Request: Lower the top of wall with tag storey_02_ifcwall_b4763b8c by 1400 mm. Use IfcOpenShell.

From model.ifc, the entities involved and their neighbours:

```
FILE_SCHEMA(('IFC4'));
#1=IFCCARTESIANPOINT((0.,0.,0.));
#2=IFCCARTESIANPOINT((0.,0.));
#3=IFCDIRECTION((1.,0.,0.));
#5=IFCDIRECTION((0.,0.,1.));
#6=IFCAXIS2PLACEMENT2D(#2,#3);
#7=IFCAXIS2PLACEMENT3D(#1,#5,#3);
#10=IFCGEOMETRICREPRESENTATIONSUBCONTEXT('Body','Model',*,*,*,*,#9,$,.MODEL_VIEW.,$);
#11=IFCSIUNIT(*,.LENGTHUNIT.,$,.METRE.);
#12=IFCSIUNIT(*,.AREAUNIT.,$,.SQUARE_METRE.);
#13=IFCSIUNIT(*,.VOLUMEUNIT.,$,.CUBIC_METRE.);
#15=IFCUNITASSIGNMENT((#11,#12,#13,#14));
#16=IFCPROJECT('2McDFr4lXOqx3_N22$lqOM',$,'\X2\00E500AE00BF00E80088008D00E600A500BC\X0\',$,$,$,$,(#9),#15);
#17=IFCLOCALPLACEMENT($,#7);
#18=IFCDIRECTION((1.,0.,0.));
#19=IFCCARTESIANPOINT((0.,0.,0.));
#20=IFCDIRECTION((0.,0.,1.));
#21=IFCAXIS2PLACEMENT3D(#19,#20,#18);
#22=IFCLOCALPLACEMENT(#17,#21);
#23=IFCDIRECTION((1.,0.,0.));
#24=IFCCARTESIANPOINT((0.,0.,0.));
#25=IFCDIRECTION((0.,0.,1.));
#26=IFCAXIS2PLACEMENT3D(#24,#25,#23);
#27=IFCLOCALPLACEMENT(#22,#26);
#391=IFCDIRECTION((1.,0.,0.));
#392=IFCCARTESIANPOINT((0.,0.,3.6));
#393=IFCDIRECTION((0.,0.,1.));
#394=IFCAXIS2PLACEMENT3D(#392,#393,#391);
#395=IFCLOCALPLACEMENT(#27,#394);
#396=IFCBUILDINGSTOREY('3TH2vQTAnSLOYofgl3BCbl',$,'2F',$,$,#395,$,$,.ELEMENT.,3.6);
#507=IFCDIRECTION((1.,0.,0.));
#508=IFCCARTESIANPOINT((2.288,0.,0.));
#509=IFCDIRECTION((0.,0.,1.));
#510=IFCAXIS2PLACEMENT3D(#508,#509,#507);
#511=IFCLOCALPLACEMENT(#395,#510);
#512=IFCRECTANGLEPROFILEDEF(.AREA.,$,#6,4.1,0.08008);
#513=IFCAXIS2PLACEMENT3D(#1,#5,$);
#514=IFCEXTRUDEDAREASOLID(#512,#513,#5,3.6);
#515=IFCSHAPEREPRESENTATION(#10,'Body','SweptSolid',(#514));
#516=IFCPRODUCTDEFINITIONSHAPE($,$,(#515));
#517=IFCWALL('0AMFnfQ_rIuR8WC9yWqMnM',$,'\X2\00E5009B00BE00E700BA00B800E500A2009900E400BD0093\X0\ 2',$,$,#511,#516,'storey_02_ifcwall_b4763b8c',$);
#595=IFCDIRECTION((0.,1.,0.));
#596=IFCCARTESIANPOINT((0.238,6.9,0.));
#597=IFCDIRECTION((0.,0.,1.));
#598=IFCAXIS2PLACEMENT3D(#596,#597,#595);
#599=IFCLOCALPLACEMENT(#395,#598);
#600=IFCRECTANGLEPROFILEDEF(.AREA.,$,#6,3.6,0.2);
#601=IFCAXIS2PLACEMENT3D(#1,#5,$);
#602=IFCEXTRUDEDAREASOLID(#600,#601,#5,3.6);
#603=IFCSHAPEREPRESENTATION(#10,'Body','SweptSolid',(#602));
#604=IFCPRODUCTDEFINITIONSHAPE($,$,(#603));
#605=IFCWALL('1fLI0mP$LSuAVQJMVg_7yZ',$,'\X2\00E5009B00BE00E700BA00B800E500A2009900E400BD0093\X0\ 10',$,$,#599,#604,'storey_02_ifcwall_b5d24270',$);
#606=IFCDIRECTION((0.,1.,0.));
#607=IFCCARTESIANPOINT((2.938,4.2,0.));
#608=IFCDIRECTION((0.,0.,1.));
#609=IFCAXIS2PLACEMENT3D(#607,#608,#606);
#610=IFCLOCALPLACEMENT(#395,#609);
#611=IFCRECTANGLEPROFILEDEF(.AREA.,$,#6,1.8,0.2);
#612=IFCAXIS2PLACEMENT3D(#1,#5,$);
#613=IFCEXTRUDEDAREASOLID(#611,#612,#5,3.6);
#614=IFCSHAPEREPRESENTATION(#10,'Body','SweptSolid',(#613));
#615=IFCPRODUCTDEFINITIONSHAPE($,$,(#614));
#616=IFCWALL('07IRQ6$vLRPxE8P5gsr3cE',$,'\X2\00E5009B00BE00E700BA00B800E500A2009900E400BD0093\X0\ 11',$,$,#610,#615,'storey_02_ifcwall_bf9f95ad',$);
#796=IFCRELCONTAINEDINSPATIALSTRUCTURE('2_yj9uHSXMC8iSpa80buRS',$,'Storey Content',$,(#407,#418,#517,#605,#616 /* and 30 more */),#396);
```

```python
import ifcopenshell
import ifcopenshell.geom
import ifcopenshell.util.representation
import ifcopenshell.util.shape
import ifcopenshell.util.unit

model = ifcopenshell.open("model.ifc")
unit_scale = ifcopenshell.util.unit.calculate_unit_scale(model)
settings = ifcopenshell.geom.settings()


def volume(element):
    """Net volume in cubic metres, openings subtracted."""
    shape = ifcopenshell.geom.create_shape(settings, element)
    return ifcopenshell.util.shape.get_volume(shape.geometry)


wall = model.by_guid("0AMFnfQ_rIuR8WC9yWqMnM")
before = volume(wall)

body = ifcopenshell.util.representation.get_representation(wall, "Model", "Body")
solid = body.Items[0]
old_height = solid.Depth
solid.Depth -= 1.4 / unit_scale
after = volume(wall)

print(f"height {old_height:g} -> {solid.Depth:g}, volume {before:.3f} -> {after:.3f} m3")

model.write("model-out.ifc")
```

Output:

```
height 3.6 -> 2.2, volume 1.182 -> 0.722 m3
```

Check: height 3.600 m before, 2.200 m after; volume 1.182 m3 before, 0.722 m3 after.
